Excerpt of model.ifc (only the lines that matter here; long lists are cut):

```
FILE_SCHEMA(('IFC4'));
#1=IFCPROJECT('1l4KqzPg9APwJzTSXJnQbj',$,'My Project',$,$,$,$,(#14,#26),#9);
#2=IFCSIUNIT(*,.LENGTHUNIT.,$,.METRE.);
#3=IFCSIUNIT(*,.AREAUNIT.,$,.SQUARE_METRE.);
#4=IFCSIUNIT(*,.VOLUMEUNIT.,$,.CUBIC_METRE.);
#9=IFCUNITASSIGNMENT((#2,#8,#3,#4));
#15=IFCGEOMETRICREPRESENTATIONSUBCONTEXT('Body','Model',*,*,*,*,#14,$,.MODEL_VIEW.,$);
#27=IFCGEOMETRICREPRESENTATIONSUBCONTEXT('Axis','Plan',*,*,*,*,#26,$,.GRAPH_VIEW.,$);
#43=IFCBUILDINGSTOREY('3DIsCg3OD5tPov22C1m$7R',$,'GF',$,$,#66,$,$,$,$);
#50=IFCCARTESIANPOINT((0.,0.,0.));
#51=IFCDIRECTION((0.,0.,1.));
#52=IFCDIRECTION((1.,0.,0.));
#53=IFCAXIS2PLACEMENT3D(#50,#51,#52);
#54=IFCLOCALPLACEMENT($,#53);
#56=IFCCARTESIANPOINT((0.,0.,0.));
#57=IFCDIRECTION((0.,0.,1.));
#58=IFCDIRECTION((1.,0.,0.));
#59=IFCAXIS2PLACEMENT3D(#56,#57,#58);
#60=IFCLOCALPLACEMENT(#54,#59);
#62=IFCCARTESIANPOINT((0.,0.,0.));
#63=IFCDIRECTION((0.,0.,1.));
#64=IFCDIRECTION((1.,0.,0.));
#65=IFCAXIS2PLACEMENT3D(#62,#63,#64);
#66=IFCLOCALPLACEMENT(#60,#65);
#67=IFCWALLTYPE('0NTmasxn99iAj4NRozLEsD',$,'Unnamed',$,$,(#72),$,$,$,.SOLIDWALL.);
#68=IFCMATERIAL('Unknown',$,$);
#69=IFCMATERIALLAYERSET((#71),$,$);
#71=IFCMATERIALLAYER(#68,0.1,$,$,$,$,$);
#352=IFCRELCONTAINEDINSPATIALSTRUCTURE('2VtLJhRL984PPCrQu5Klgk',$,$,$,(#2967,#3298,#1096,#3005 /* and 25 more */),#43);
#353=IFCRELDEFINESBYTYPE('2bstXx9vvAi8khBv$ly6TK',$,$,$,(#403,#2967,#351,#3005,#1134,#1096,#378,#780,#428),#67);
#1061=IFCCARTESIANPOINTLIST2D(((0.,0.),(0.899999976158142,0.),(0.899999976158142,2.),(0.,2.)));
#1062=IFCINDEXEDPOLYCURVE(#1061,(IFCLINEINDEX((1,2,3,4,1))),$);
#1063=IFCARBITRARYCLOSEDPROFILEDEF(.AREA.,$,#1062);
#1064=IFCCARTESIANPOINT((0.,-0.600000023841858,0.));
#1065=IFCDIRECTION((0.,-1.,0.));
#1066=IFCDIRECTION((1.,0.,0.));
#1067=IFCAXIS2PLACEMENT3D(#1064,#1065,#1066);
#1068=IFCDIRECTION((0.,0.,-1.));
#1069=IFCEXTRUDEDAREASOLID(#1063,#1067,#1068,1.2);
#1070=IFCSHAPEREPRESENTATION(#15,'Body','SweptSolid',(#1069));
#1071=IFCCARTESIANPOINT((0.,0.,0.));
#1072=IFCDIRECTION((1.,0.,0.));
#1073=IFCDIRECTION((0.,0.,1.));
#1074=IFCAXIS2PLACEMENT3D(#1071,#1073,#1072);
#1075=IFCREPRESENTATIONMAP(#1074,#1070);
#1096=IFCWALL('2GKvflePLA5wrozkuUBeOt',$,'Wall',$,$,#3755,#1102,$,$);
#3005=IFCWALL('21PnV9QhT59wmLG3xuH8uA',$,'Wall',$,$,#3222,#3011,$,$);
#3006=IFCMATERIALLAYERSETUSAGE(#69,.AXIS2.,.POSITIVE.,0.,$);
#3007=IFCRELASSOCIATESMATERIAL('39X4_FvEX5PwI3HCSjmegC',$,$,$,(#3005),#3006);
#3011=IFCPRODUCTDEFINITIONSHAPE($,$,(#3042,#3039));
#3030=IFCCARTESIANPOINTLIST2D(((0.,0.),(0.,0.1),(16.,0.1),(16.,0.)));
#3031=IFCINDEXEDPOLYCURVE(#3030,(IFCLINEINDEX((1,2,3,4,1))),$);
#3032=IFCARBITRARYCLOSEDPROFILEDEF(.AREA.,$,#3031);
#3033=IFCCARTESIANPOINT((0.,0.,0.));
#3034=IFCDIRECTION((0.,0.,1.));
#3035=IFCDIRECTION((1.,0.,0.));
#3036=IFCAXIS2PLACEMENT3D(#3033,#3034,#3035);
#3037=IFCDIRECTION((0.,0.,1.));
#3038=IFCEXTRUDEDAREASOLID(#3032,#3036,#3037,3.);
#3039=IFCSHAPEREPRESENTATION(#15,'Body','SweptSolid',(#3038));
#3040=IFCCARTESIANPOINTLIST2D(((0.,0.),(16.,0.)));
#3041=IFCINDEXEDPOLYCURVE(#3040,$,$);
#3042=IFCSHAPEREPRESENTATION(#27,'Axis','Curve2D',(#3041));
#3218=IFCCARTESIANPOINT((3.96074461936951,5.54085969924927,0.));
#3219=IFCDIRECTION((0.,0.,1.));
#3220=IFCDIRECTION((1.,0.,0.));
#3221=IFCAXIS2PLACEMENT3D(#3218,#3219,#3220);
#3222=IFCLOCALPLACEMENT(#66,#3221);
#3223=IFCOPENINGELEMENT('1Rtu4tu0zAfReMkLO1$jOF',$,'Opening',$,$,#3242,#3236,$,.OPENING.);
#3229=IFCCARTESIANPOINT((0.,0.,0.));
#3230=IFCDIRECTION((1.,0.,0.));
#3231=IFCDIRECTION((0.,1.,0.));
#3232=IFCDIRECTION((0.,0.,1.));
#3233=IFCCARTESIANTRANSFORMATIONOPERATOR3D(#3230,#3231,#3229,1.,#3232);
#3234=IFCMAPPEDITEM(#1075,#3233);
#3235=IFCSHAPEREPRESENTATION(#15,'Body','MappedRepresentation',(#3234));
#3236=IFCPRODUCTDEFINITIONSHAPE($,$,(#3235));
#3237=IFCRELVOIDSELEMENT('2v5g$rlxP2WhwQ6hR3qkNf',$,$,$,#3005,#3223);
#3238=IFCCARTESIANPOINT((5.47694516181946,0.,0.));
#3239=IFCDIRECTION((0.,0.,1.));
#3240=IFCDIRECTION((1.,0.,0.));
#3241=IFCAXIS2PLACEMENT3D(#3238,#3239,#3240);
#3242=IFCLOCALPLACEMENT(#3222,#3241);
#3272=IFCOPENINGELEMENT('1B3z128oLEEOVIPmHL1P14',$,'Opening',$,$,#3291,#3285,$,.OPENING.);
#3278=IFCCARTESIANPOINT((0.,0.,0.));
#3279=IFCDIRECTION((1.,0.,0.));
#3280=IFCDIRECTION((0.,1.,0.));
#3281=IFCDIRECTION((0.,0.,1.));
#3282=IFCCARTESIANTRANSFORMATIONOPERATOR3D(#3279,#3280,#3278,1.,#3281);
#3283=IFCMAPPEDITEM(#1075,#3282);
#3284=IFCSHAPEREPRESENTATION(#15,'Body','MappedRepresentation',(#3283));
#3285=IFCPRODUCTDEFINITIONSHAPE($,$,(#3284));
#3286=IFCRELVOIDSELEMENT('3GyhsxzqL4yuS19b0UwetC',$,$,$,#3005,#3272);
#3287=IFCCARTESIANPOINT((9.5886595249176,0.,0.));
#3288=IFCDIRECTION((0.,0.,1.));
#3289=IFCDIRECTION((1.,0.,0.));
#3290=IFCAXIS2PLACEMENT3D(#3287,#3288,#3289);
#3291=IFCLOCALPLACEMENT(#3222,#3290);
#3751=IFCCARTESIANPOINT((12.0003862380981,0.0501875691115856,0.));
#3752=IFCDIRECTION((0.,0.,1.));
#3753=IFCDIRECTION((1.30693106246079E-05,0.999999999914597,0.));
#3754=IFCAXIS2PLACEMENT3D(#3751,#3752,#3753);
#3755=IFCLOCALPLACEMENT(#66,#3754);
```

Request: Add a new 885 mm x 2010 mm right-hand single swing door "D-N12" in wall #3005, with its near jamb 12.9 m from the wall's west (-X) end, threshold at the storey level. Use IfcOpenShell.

```python
import numpy as np
import ifcopenshell
import ifcopenshell.api.feature
import ifcopenshell.api.geometry
import ifcopenshell.api.root
import ifcopenshell.api.spatial
import ifcopenshell.geom
import ifcopenshell.util.element
import ifcopenshell.util.placement
import ifcopenshell.util.representation
import ifcopenshell.util.shape
import ifcopenshell.util.unit

model = ifcopenshell.open("model.ifc")
unit_scale = ifcopenshell.util.unit.calculate_unit_scale(model)
settings = ifcopenshell.geom.settings()


def volume(element):
    """Net volume in cubic metres, openings subtracted."""
    shape = ifcopenshell.geom.create_shape(settings, element)
    return ifcopenshell.util.shape.get_volume(shape.geometry)


wall = model.by_guid("21PnV9QhT59wmLG3xuH8uA")
storey = ifcopenshell.util.element.get_container(wall, ifc_class="IfcBuildingStorey")
context = ifcopenshell.util.representation.get_context(model, "Model", "Body", "MODEL_VIEW")
before = volume(wall)

width, height, from_end, sill = 0.885, 2.01, 12.9, 0.0  # metres

# The wall runs along its own X axis, and the end named is its -X end.
wall_shape = ifcopenshell.geom.create_shape(settings, wall)
x, y, z = ifcopenshell.util.shape.get_vertices(wall_shape.geometry).T
start = x.min() + from_end
face, thickness = float(y.min()), float(y.max() - y.min())
wall_matrix = ifcopenshell.util.placement.get_local_placement(wall.ObjectPlacement)
level = ifcopenshell.util.placement.get_local_placement(storey.ObjectPlacement)[2, 3]


def in_wall(x, y):
    """Placement at x, y metres in the wall's axes, at sill height."""
    matrix = wall_matrix.copy()
    matrix[:, 3] = wall_matrix @ np.array([x / unit_scale, y / unit_scale, 0.0, 1.0])
    matrix[2, 3] = level + sill / unit_scale
    return matrix


# Opening: a box that overshoots both wall faces by 50 mm.
opening = ifcopenshell.api.root.create_entity(model, ifc_class="IfcOpeningElement", predefined_type="OPENING")
box = ifcopenshell.api.geometry.add_wall_representation(
    model, context=context, length=width, height=height, thickness=thickness + 0.1
)
ifcopenshell.api.geometry.assign_representation(model, product=opening, representation=box)
ifcopenshell.api.geometry.edit_object_placement(model, product=opening, matrix=in_wall(start, face - 0.05), is_si=False)
ifcopenshell.api.feature.add_feature(model, feature=opening, element=wall)

door = ifcopenshell.api.root.create_entity(model, ifc_class="IfcDoor", name="D-N12", predefined_type="DOOR")
door.OverallWidth, door.OverallHeight = width / unit_scale, height / unit_scale
door.OperationType = "SINGLE_SWING_RIGHT"
body = ifcopenshell.api.geometry.add_door_representation(
    model,
    context=context,
    overall_width=door.OverallWidth,
    overall_height=door.OverallHeight,
    operation_type="SINGLE_SWING_RIGHT",
    lining_properties={"LiningDepth": thickness / unit_scale, "ThresholdDepth": thickness / unit_scale},
)
ifcopenshell.api.geometry.assign_representation(model, product=door, representation=body)
ifcopenshell.api.spatial.assign_container(model, products=[door], relating_structure=storey)
ifcopenshell.api.feature.add_filling(model, opening=opening, element=door)

# The lining spans the wall, so the door starts at the wall face.
ifcopenshell.api.geometry.edit_object_placement(model, product=door, matrix=in_wall(start, face), is_si=False)

after = volume(wall)

print(f"wall volume {before:.3f} -> {after:.3f} m3")

model.write("model-out.ifc")
```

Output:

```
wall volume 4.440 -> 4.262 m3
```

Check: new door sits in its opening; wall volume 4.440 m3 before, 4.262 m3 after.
